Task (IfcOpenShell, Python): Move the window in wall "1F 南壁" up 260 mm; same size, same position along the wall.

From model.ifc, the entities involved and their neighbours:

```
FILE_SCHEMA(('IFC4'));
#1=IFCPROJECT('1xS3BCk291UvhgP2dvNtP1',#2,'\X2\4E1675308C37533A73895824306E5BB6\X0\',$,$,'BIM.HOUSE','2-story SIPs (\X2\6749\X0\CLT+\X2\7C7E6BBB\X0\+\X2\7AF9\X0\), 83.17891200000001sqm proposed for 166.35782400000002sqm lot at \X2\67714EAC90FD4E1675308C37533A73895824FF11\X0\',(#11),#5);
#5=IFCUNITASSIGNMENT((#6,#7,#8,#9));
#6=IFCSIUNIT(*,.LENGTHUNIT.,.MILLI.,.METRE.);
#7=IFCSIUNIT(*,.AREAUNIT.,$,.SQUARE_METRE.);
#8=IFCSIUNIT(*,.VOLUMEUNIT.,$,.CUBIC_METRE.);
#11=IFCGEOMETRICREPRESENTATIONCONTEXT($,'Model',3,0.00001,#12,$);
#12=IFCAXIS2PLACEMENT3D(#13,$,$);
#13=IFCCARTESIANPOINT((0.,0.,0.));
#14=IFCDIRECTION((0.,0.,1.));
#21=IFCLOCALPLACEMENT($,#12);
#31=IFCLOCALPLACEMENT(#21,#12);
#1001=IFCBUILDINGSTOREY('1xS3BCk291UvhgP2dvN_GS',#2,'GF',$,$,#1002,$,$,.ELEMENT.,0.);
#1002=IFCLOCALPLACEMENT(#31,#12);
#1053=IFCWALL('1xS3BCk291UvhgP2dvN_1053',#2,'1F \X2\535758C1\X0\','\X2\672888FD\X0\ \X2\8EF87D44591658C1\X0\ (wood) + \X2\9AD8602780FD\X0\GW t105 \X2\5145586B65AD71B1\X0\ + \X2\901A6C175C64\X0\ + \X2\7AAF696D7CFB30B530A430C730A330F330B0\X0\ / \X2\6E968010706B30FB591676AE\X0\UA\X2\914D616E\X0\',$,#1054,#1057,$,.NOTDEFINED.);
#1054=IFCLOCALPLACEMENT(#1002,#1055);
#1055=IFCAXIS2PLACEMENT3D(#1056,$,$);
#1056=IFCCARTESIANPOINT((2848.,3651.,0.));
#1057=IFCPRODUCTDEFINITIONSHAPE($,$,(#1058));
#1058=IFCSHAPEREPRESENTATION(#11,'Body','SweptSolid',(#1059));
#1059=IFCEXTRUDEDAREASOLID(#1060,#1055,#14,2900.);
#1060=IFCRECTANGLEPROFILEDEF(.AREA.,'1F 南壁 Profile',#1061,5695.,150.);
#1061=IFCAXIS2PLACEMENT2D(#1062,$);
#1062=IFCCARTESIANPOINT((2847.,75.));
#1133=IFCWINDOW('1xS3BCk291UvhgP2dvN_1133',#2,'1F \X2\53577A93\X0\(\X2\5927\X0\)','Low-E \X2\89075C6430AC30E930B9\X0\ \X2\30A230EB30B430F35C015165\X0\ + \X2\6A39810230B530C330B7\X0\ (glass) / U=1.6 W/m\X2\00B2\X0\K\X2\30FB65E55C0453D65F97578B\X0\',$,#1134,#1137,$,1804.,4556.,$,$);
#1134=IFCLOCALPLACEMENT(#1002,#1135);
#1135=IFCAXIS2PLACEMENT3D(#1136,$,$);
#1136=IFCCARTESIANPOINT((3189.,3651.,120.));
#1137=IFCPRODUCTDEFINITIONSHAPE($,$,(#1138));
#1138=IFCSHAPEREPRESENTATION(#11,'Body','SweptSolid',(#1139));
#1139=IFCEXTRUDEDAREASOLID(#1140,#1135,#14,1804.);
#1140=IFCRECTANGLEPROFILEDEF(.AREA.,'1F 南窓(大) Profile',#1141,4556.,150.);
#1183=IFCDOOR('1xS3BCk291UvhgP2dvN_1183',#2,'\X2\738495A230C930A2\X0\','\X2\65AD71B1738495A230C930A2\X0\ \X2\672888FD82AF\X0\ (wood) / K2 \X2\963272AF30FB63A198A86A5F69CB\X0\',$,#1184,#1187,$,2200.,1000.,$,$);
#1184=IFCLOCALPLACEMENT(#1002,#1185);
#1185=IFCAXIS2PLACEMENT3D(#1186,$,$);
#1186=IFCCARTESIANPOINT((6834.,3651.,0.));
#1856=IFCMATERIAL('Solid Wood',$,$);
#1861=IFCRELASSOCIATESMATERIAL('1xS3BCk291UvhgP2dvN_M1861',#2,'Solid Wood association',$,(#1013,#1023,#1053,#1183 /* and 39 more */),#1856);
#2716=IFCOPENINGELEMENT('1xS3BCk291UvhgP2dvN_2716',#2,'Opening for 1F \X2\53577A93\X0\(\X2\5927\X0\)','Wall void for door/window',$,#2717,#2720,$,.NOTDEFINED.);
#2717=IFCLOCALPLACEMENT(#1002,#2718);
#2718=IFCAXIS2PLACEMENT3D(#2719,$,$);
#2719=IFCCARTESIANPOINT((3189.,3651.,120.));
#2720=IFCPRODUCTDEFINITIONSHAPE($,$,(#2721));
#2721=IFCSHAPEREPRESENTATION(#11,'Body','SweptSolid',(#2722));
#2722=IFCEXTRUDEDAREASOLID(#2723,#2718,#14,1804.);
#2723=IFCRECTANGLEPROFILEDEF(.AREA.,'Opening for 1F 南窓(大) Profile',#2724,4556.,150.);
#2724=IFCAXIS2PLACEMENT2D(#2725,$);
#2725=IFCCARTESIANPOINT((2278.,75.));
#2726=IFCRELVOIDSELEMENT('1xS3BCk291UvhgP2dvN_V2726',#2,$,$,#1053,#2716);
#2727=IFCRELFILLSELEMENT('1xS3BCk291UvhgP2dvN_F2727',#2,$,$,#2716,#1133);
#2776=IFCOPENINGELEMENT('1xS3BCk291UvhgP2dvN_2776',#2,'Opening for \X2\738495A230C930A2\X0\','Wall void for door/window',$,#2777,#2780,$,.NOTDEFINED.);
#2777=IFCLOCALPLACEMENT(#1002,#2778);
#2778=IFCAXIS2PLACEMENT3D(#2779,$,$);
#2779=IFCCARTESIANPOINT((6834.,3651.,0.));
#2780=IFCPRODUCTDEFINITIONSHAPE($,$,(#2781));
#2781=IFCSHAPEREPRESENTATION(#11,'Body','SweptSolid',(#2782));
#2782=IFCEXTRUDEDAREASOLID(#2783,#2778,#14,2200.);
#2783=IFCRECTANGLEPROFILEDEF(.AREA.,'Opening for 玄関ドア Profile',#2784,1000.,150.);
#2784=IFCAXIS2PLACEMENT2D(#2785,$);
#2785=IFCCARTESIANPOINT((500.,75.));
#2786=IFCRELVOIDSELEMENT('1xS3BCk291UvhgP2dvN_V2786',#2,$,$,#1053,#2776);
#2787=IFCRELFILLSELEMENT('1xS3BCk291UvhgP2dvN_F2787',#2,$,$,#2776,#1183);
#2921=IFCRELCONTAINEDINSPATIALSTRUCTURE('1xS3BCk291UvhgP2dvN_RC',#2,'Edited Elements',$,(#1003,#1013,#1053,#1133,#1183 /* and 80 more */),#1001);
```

```python
import numpy as np
import ifcopenshell
import ifcopenshell.api.geometry
import ifcopenshell.util.placement
import ifcopenshell.util.unit

model = ifcopenshell.open("model.ifc")
unit_scale = ifcopenshell.util.unit.calculate_unit_scale(model)

window = model.by_guid("1xS3BCk291UvhgP2dvN_1133")
opening = window.FillsVoids[0].RelatingOpeningElement
dz = 0.26 / unit_scale

shift = np.array([0.0, 0.0, dz])
# The window is not placed relative to its opening, so move both.
for product in (opening, window):
    matrix = ifcopenshell.util.placement.get_local_placement(product.ObjectPlacement)
    matrix[:3, 3] += shift
    ifcopenshell.api.geometry.edit_object_placement(model, product=product, matrix=matrix, is_si=False)

print(f"moved by {dz * unit_scale:+.3f} m")

model.write("model_updated.ifc")
```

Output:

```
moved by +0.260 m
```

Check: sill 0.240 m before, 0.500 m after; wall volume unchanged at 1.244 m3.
